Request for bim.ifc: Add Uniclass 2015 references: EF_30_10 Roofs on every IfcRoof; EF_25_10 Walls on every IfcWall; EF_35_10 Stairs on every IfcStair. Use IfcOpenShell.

First a look at what the model holds.

```python
import ifcopenshell

model = ifcopenshell.open("bim.ifc")
print(model.schema)
print("classifications:", [c.Name for c in model.by_type("IfcClassification")])
for ifc_class in ("IfcDoor", "IfcRoof", "IfcStair", "IfcWall", "IfcWindow"):
    print(ifc_class, len(model.by_type(ifc_class)))
```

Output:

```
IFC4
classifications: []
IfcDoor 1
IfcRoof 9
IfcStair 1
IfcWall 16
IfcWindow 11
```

```python
import ifcopenshell
import ifcopenshell.api.classification

model = ifcopenshell.open("bim.ifc")

system = ifcopenshell.api.classification.add_classification(model, classification="Uniclass 2015")

codes = {
    "IfcRoof": ("EF_30_10", "Roofs"),
    "IfcWall": ("EF_25_10", "Walls"),
    "IfcStair": ("EF_35_10", "Stairs"),
}
for ifc_class, (code, name) in codes.items():
    products = model.by_type(ifc_class)
    ifcopenshell.api.classification.add_reference(
        model, products=products, classification=system, identification=code, name=name
    )
    print(code, len(products))

model.write("bim-out.ifc")
```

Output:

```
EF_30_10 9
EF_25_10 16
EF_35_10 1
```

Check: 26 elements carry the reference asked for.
